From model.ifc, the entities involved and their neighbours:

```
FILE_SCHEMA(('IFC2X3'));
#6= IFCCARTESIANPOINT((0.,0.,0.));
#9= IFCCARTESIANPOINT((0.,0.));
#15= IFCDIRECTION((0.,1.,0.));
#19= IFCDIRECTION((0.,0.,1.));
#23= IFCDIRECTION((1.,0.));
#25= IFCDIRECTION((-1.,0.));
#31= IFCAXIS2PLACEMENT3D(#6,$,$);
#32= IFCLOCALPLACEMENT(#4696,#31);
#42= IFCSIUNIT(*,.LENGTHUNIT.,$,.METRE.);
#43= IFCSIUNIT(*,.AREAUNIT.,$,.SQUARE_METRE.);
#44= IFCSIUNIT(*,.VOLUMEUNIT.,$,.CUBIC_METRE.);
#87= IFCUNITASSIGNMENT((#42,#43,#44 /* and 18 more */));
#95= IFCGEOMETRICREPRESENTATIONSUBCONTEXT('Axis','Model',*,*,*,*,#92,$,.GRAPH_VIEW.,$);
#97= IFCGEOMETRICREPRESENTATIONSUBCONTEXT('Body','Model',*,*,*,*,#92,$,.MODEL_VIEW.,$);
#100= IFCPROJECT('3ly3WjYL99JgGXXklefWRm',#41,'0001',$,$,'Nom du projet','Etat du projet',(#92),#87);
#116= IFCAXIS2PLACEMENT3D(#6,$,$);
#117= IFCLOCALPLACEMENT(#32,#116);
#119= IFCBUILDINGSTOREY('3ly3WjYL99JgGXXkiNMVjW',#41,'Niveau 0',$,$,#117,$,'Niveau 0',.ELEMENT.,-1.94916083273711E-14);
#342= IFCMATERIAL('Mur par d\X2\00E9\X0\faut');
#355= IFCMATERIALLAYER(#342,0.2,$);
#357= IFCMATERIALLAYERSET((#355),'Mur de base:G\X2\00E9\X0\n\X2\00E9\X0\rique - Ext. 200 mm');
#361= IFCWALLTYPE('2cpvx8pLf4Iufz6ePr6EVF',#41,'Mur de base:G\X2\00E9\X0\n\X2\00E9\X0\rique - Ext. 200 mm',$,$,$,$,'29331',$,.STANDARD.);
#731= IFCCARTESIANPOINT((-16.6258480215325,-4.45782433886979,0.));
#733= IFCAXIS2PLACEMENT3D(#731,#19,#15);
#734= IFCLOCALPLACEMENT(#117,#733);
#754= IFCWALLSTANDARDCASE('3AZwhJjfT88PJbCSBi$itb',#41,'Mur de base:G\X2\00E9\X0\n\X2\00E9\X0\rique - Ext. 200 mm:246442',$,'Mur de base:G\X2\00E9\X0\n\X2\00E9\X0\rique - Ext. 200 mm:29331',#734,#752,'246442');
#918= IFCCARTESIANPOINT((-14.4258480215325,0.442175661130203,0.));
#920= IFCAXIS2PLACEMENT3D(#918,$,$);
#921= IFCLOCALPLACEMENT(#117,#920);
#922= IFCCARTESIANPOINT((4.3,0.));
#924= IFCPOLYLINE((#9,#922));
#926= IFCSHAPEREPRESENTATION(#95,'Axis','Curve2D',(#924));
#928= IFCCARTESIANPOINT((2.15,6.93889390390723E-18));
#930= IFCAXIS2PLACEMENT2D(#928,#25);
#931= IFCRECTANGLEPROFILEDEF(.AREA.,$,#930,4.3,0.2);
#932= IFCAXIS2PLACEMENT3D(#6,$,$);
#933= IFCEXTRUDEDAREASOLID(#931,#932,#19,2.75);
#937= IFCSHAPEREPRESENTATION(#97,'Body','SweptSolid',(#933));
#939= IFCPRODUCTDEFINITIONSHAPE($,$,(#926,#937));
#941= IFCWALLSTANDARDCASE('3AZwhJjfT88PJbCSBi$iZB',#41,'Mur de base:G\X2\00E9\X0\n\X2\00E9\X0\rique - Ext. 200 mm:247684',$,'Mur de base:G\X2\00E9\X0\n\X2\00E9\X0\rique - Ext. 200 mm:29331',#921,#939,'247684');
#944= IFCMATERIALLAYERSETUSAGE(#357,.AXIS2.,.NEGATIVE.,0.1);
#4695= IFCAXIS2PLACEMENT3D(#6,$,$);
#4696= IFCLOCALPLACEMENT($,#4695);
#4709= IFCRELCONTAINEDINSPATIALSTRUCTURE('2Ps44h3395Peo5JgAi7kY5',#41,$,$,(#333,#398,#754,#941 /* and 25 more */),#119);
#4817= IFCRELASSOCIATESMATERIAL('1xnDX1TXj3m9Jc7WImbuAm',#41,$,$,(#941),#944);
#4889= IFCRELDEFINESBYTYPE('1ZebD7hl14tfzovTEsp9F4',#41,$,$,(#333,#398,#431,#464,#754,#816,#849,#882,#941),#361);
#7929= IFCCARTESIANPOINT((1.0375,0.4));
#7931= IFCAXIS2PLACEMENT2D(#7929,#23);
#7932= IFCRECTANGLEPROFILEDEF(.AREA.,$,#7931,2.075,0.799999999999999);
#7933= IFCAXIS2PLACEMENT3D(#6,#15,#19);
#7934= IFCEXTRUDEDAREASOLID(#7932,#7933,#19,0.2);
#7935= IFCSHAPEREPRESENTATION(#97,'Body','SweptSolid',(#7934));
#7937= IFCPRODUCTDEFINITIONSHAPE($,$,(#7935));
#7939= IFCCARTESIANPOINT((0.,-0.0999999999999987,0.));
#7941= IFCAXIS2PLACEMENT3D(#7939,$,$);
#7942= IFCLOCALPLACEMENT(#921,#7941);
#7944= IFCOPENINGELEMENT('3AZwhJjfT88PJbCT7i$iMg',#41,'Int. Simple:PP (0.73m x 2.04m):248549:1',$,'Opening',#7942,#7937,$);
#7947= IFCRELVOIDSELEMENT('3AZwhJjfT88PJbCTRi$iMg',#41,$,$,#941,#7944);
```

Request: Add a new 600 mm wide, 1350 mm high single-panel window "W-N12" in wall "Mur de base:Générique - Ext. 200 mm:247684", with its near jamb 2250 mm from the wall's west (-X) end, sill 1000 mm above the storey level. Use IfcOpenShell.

```python
import numpy as np
import ifcopenshell
import ifcopenshell.api.feature
import ifcopenshell.api.geometry
import ifcopenshell.api.root
import ifcopenshell.api.spatial
import ifcopenshell.api.type
import ifcopenshell.geom
import ifcopenshell.util.element
import ifcopenshell.util.placement
import ifcopenshell.util.representation
import ifcopenshell.util.shape
import ifcopenshell.util.unit

model = ifcopenshell.open("model.ifc")
unit_scale = ifcopenshell.util.unit.calculate_unit_scale(model)
settings = ifcopenshell.geom.settings()


def volume(element):
    """Net volume in cubic metres, openings subtracted."""
    shape = ifcopenshell.geom.create_shape(settings, element)
    return ifcopenshell.util.shape.get_volume(shape.geometry)


wall = model.by_guid("3AZwhJjfT88PJbCSBi$iZB")
storey = ifcopenshell.util.element.get_container(wall, ifc_class="IfcBuildingStorey")
context = ifcopenshell.util.representation.get_context(model, "Model", "Body", "MODEL_VIEW")
before = volume(wall)

width, height, from_end, sill = 0.6, 1.35, 2.25, 1  # metres

# The wall runs along its own X axis, and the end named is its -X end.
wall_shape = ifcopenshell.geom.create_shape(settings, wall)
x, y, z = ifcopenshell.util.shape.get_vertices(wall_shape.geometry).T
start = x.min() + from_end
face, thickness = float(y.min()), float(y.max() - y.min())
wall_matrix = ifcopenshell.util.placement.get_local_placement(wall.ObjectPlacement)
level = ifcopenshell.util.placement.get_local_placement(storey.ObjectPlacement)[2, 3]


def in_wall(x, y):
    """Placement at x, y metres in the wall's axes, at sill height."""
    matrix = wall_matrix.copy()
    matrix[:, 3] = wall_matrix @ np.array([x / unit_scale, y / unit_scale, 0.0, 1.0])
    matrix[2, 3] = level + sill / unit_scale
    return matrix


# Opening: a box that overshoots both wall faces by 50 mm.
opening = ifcopenshell.api.root.create_entity(model, ifc_class="IfcOpeningElement")
box = ifcopenshell.api.geometry.add_wall_representation(
    model, context=context, length=width, height=height, thickness=thickness + 0.1
)
ifcopenshell.api.geometry.assign_representation(model, product=opening, representation=box)
ifcopenshell.api.geometry.edit_object_placement(model, product=opening, matrix=in_wall(start, face - 0.05), is_si=False)
ifcopenshell.api.feature.add_feature(model, feature=opening, element=wall)

window = ifcopenshell.api.root.create_entity(model, ifc_class="IfcWindow", name="W-N12")
window.OverallWidth, window.OverallHeight = width / unit_scale, height / unit_scale
body = ifcopenshell.api.geometry.add_window_representation(
    model,
    context=context,
    overall_width=window.OverallWidth,
    overall_height=window.OverallHeight,
    partition_type="SINGLE_PANEL",
)
ifcopenshell.api.geometry.assign_representation(model, product=window, representation=body)
ifcopenshell.api.spatial.assign_container(model, products=[window], relating_structure=storey)
fills = ifcopenshell.api.feature.add_filling(model, opening=opening, element=window)
fills.OwnerHistory = window.OwnerHistory  # required in IFC2X3

# IFC2X3 keeps the operation on the window style.
style = ifcopenshell.api.root.create_entity(model, ifc_class="IfcWindowStyle", name="W-N12")
style.OperationType, style.ConstructionType = "SINGLE_PANEL", "NOTDEFINED"
style.ParameterTakesPrecedence = style.Sizeable = False
ifcopenshell.api.type.assign_type(model, related_objects=[window], relating_type=style)

# Centre the window in the wall's thickness.
ifcopenshell.api.geometry.edit_object_placement(model, product=window, matrix=in_wall(start, face), is_si=False)
window_shape = ifcopenshell.geom.create_shape(settings, window)
depth = ifcopenshell.util.shape.get_vertices(window_shape.geometry)[:, 1]
offset = face + thickness / 2 - (depth.min() + depth.max()) / 2
ifcopenshell.api.geometry.edit_object_placement(model, product=window, matrix=in_wall(start, offset), is_si=False)

after = volume(wall)

print(f"wall volume {before:.3f} -> {after:.3f} m3")

model.write("model_rev.ifc")
```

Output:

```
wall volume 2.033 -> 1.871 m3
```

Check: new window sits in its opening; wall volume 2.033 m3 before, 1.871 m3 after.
